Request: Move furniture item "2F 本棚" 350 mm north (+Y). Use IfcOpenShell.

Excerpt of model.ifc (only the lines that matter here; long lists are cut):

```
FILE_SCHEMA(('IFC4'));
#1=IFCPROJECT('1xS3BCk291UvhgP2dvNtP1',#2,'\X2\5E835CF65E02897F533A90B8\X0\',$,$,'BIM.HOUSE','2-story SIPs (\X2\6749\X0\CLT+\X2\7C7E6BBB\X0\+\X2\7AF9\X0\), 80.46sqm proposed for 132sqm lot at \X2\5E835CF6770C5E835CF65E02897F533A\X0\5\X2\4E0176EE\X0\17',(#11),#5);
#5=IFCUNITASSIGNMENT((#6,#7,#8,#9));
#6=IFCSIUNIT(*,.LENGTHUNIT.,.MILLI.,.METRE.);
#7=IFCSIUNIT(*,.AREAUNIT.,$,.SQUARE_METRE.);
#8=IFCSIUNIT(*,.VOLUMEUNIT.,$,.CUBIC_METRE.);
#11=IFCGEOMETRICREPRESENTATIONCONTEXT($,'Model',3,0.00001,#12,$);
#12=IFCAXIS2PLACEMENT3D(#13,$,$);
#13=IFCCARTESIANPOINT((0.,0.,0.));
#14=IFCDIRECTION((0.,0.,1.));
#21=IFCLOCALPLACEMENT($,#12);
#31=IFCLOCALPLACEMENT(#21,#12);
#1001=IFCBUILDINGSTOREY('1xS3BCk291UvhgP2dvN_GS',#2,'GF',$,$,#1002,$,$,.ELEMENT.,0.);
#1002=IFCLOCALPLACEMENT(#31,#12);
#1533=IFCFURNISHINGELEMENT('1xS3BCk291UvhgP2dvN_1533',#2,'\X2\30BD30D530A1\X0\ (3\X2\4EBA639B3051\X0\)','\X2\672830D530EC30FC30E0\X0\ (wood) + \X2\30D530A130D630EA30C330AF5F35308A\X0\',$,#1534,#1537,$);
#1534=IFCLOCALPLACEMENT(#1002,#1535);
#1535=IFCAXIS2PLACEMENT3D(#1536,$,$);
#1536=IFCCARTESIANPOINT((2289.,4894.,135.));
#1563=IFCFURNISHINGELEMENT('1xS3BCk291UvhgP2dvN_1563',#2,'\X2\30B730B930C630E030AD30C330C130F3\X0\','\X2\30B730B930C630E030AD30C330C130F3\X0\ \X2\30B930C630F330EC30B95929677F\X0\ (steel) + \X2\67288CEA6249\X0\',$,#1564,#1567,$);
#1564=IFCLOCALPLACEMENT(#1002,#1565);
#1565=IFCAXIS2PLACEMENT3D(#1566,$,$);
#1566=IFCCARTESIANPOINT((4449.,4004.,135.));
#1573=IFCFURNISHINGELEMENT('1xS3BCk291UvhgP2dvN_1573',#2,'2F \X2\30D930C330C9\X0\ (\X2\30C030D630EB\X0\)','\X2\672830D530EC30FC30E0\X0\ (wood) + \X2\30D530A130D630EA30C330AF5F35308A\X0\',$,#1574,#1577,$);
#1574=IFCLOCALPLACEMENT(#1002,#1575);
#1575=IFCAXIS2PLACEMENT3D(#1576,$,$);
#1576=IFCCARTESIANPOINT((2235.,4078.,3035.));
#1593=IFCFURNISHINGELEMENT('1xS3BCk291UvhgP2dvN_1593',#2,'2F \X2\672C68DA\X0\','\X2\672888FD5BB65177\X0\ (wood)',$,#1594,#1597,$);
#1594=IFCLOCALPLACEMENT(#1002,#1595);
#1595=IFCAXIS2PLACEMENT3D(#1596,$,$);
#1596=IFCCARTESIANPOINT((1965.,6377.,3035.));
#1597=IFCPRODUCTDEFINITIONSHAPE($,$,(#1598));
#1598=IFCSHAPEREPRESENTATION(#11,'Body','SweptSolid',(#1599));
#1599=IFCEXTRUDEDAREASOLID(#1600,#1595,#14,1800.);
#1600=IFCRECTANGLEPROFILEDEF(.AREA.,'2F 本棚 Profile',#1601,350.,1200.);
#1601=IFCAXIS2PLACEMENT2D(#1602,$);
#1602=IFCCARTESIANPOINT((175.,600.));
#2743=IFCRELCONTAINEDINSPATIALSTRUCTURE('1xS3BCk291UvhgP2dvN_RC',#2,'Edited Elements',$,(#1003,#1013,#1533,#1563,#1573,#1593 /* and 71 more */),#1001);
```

```python
import ifcopenshell
import ifcopenshell.api.geometry
import ifcopenshell.util.placement

model = ifcopenshell.open("model.ifc")

item = model.by_guid("1xS3BCk291UvhgP2dvN_1593")
matrix = ifcopenshell.util.placement.get_local_placement(item.ObjectPlacement)
matrix[1, 3] += 350.0
ifcopenshell.api.geometry.edit_object_placement(model, product=item, matrix=matrix, is_si=False)

print(ifcopenshell.util.placement.get_local_placement(item.ObjectPlacement).round(3) + 0.0)

model.write("model-out.ifc")
```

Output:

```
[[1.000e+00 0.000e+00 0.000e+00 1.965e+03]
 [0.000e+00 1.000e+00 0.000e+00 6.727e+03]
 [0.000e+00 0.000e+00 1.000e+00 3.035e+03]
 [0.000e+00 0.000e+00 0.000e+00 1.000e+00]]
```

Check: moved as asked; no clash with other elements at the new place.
